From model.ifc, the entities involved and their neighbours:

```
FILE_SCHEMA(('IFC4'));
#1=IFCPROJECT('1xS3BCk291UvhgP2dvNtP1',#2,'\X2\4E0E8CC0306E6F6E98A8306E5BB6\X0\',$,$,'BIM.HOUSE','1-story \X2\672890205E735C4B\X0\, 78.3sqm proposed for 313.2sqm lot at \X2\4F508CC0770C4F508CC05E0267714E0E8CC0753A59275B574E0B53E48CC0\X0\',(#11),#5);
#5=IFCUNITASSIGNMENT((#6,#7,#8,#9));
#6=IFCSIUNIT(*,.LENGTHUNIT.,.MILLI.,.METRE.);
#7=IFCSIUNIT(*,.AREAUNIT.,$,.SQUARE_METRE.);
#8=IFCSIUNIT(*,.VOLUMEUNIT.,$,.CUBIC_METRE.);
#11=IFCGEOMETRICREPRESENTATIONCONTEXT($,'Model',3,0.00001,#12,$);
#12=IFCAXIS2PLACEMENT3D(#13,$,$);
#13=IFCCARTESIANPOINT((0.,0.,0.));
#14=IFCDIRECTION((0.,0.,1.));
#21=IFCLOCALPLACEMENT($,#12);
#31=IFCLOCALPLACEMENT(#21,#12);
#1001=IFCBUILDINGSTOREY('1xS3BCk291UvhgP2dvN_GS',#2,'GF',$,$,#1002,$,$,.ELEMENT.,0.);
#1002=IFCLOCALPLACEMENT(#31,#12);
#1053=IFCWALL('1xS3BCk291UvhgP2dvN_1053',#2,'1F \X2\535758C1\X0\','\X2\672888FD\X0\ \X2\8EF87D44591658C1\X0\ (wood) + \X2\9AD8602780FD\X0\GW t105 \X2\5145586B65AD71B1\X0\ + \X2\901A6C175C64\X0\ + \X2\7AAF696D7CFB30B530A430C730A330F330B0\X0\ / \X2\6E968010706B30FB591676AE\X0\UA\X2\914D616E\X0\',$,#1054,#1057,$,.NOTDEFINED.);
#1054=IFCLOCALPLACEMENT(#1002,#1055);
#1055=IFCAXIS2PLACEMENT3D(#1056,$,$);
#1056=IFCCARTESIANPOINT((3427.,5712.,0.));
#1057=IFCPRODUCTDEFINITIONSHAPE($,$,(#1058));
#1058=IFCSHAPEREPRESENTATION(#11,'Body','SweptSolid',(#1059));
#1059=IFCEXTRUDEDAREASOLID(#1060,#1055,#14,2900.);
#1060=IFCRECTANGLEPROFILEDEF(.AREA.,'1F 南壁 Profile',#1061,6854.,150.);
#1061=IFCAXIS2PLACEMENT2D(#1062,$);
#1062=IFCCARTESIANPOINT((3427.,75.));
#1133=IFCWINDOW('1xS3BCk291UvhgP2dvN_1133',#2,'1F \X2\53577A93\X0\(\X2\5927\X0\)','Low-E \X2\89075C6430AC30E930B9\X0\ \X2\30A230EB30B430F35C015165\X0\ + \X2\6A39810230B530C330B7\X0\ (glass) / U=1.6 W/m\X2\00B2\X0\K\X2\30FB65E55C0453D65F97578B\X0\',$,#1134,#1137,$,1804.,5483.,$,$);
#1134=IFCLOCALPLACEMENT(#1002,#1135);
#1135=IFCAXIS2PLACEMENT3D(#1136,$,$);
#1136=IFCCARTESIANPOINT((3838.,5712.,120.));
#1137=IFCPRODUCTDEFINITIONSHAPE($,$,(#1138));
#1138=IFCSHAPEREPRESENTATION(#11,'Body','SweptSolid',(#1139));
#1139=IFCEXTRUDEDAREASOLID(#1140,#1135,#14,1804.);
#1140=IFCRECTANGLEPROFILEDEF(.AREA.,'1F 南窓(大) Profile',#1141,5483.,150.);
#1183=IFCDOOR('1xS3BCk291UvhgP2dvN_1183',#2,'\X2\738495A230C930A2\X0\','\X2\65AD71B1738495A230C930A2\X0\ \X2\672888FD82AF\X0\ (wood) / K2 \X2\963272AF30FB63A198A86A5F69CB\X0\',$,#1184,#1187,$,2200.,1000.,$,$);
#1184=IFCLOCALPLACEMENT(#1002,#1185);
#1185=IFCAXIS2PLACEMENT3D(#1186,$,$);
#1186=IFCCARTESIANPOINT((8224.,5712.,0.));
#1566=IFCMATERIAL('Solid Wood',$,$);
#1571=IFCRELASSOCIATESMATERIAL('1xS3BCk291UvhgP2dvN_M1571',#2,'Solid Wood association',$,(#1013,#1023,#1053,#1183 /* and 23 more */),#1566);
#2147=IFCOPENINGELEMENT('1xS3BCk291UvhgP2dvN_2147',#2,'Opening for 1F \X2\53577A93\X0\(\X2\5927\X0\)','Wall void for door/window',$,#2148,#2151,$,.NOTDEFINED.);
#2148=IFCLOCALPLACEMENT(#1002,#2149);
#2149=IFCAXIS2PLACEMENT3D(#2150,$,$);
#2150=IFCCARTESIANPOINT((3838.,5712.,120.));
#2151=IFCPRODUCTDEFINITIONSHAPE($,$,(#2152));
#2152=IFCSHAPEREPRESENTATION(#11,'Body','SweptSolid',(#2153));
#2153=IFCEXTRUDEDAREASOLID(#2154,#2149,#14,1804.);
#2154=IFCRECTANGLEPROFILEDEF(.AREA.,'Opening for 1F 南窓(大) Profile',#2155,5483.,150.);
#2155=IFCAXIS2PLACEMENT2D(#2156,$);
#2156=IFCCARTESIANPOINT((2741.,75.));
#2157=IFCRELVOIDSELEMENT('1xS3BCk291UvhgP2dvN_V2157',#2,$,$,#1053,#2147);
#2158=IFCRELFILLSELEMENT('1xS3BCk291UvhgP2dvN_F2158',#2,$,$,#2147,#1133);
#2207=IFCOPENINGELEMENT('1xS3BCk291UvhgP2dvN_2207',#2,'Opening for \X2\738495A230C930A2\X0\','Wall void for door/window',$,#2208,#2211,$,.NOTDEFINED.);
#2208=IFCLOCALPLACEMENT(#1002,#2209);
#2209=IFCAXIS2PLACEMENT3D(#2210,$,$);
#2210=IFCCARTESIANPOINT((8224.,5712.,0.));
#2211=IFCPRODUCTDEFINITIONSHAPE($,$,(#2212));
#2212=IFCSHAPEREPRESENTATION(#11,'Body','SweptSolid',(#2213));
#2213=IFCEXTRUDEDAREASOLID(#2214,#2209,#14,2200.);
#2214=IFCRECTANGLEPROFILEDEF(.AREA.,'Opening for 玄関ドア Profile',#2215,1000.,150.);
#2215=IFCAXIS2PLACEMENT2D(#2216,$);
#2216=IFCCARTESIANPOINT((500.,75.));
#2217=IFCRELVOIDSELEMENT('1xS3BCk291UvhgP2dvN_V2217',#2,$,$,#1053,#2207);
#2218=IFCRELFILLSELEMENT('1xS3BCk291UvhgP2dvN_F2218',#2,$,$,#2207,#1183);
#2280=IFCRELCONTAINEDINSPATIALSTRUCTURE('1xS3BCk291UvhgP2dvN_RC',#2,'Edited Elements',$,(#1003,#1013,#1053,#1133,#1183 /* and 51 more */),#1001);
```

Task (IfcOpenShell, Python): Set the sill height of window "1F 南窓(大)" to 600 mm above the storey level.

```python
import numpy as np
import ifcopenshell
import ifcopenshell.api.geometry
import ifcopenshell.geom
import ifcopenshell.util.element
import ifcopenshell.util.placement
import ifcopenshell.util.shape
import ifcopenshell.util.unit

model = ifcopenshell.open("model.ifc")
unit_scale = ifcopenshell.util.unit.calculate_unit_scale(model)

window = model.by_guid("1xS3BCk291UvhgP2dvN_1133")
opening = window.FillsVoids[0].RelatingOpeningElement
storey = ifcopenshell.util.element.get_container(window, ifc_class="IfcBuildingStorey")
level = ifcopenshell.util.placement.get_local_placement(storey.ObjectPlacement)[2, 3]

# The opening's origin need not be at the sill, so measure its lowest point.
shape = ifcopenshell.geom.create_shape(ifcopenshell.geom.settings(), opening)
bottom = ifcopenshell.util.shape.get_shape_bottom_elevation(shape, shape.geometry) / unit_scale
dz = level + 0.6 / unit_scale - bottom

shift = np.array([0.0, 0.0, dz])
# The window is not placed relative to its opening, so move both.
for product in (opening, window):
    matrix = ifcopenshell.util.placement.get_local_placement(product.ObjectPlacement)
    matrix[:3, 3] += shift
    ifcopenshell.api.geometry.edit_object_placement(model, product=product, matrix=matrix, is_si=False)

print(f"moved by {dz * unit_scale:+.3f} m")

model.write("model_updated.ifc")
```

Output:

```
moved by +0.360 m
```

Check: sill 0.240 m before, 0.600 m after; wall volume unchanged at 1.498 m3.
